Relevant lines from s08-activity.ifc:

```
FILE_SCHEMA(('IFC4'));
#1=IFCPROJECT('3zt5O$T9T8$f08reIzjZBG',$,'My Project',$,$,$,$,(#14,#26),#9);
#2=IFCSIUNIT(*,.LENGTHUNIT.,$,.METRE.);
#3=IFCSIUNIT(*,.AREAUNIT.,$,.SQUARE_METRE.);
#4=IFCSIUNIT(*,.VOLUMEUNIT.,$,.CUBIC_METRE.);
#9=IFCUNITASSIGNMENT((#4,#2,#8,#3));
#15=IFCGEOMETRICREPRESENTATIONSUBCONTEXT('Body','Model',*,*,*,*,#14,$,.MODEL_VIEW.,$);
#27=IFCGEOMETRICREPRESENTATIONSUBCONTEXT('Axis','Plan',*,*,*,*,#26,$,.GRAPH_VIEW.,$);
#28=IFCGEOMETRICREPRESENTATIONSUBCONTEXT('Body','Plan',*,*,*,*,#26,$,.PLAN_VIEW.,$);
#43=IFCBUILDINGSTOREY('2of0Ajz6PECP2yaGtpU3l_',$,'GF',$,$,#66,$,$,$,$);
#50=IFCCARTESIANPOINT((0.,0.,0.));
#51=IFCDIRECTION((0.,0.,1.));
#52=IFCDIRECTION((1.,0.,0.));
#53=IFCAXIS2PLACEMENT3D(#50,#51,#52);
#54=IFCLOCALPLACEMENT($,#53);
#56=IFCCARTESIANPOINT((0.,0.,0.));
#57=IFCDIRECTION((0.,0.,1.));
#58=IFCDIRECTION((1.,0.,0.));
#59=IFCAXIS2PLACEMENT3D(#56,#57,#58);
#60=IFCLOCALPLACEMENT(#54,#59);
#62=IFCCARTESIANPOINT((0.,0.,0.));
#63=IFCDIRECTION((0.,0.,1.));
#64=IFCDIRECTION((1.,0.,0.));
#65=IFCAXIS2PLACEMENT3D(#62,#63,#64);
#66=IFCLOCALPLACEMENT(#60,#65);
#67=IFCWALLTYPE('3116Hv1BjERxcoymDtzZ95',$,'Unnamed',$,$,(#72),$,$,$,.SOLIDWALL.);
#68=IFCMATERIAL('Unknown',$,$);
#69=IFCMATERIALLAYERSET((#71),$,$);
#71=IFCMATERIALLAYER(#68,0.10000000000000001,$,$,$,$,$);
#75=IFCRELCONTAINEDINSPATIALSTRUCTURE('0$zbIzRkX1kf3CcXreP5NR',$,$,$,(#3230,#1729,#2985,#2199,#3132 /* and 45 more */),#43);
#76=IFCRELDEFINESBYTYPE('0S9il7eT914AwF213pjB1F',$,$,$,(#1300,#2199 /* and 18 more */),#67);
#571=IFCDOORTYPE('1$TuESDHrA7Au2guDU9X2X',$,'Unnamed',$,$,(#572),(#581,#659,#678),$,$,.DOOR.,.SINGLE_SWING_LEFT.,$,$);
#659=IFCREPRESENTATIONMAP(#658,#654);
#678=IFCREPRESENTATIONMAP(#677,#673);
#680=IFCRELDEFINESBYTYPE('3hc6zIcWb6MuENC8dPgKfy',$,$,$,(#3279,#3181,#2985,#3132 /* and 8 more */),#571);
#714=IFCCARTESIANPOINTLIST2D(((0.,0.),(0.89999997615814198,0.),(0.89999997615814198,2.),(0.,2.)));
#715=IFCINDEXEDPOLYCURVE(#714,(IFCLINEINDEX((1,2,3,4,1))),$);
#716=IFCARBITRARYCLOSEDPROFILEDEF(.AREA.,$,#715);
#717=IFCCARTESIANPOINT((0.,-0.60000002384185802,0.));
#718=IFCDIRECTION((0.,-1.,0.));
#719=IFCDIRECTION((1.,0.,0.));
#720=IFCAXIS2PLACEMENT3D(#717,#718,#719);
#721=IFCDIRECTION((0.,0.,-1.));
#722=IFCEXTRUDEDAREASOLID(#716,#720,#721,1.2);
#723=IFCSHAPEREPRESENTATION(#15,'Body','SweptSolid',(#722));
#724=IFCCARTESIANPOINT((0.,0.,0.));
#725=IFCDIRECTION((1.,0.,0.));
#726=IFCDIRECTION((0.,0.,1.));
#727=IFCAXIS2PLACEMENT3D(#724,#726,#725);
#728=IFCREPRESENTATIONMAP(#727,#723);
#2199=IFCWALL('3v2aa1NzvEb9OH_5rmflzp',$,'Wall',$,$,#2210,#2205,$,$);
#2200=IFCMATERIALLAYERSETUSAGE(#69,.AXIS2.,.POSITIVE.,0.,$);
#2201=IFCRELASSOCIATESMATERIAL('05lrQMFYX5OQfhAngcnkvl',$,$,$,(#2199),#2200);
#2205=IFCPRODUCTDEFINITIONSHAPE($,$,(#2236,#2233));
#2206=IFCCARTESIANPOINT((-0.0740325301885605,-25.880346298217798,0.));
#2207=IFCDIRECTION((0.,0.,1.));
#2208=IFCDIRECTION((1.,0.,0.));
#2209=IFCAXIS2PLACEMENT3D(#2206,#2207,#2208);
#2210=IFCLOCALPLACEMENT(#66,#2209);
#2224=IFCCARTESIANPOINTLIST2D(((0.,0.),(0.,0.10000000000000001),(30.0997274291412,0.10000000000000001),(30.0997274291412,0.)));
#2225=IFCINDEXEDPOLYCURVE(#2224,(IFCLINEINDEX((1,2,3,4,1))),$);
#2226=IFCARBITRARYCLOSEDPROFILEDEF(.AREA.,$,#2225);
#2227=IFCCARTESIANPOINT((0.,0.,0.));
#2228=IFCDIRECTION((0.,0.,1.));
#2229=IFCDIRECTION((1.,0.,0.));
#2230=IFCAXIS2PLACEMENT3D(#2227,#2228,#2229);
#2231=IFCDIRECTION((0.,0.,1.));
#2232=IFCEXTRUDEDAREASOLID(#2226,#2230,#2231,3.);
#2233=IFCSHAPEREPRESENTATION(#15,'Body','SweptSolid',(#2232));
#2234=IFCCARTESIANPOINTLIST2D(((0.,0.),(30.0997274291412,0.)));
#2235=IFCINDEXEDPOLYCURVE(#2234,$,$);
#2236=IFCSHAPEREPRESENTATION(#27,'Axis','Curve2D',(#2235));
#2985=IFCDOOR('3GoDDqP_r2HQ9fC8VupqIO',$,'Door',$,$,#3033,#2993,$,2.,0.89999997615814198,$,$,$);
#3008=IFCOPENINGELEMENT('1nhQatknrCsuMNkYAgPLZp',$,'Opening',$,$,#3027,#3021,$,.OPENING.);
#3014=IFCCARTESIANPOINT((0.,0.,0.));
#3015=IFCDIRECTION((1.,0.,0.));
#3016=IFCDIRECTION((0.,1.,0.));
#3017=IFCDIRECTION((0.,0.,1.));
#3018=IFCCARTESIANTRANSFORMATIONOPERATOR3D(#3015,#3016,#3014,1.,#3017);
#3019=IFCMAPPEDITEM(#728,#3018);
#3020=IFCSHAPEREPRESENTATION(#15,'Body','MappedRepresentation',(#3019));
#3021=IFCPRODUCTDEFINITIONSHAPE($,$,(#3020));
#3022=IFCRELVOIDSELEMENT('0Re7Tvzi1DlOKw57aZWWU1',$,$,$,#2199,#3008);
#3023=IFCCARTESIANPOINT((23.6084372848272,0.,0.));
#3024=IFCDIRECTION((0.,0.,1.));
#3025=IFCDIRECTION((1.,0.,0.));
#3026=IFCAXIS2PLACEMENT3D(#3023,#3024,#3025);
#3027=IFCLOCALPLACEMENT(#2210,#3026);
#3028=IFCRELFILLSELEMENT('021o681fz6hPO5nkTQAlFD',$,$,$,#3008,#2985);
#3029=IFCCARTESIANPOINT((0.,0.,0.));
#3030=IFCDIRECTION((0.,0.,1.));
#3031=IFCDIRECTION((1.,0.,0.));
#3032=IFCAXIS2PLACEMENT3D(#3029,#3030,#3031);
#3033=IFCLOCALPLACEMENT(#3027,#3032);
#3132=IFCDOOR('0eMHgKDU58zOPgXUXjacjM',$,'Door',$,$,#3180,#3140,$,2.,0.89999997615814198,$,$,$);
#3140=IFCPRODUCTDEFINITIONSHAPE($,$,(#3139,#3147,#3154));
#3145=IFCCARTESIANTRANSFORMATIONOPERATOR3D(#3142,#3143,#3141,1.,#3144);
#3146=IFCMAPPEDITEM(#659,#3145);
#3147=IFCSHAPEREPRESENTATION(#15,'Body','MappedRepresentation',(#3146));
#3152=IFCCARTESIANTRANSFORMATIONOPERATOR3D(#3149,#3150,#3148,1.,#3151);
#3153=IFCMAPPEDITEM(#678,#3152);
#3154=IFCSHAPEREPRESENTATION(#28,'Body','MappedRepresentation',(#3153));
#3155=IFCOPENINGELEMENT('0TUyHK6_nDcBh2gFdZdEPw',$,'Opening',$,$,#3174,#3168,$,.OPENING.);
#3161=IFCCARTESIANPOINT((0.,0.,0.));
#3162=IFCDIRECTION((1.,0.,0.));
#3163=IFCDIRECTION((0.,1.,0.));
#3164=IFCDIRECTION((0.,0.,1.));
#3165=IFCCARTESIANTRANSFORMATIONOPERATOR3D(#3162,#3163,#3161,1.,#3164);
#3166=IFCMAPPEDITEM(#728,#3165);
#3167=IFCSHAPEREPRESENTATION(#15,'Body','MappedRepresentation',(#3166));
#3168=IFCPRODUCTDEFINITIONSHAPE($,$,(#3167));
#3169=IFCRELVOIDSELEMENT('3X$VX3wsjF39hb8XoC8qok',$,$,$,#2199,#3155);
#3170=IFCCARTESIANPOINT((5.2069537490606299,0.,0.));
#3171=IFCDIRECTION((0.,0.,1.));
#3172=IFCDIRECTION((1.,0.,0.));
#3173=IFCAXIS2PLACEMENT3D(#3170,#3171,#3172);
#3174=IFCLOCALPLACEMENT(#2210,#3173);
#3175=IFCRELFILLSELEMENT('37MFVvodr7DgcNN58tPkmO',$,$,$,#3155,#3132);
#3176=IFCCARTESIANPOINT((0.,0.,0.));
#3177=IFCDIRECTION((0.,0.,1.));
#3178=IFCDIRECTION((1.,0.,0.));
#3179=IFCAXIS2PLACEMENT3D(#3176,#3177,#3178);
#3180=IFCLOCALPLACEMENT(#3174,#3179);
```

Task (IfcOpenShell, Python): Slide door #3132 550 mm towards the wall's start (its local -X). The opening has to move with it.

```python
import ifcopenshell
import ifcopenshell.api.geometry
import ifcopenshell.util.placement
import ifcopenshell.util.unit

model = ifcopenshell.open("s08-activity.ifc")
unit_scale = ifcopenshell.util.unit.calculate_unit_scale(model)

door = model.by_id(3132)
opening = door.FillsVoids[0].RelatingOpeningElement
wall = opening.VoidsElements[0].RelatingBuildingElement

wall_matrix = ifcopenshell.util.placement.get_local_placement(wall.ObjectPlacement)
shift = wall_matrix[:3, 0] * -0.55 / unit_scale
before = ifcopenshell.util.placement.get_local_placement(door.ObjectPlacement)[:3, 3].copy()

# The door is placed relative to its opening, so it follows when the opening moves.
matrix = ifcopenshell.util.placement.get_local_placement(opening.ObjectPlacement)
matrix[:3, 3] += shift
ifcopenshell.api.geometry.edit_object_placement(
    model, product=opening, matrix=matrix, is_si=False, should_transform_children=True
)

after = ifcopenshell.util.placement.get_local_placement(door.ObjectPlacement)[:3, 3]
print("door moved by", (after - before).round(3) + 0.0)

model.write("s08-activity-out.ifc")
```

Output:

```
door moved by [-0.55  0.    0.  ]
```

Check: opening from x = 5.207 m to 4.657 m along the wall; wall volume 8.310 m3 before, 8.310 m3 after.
